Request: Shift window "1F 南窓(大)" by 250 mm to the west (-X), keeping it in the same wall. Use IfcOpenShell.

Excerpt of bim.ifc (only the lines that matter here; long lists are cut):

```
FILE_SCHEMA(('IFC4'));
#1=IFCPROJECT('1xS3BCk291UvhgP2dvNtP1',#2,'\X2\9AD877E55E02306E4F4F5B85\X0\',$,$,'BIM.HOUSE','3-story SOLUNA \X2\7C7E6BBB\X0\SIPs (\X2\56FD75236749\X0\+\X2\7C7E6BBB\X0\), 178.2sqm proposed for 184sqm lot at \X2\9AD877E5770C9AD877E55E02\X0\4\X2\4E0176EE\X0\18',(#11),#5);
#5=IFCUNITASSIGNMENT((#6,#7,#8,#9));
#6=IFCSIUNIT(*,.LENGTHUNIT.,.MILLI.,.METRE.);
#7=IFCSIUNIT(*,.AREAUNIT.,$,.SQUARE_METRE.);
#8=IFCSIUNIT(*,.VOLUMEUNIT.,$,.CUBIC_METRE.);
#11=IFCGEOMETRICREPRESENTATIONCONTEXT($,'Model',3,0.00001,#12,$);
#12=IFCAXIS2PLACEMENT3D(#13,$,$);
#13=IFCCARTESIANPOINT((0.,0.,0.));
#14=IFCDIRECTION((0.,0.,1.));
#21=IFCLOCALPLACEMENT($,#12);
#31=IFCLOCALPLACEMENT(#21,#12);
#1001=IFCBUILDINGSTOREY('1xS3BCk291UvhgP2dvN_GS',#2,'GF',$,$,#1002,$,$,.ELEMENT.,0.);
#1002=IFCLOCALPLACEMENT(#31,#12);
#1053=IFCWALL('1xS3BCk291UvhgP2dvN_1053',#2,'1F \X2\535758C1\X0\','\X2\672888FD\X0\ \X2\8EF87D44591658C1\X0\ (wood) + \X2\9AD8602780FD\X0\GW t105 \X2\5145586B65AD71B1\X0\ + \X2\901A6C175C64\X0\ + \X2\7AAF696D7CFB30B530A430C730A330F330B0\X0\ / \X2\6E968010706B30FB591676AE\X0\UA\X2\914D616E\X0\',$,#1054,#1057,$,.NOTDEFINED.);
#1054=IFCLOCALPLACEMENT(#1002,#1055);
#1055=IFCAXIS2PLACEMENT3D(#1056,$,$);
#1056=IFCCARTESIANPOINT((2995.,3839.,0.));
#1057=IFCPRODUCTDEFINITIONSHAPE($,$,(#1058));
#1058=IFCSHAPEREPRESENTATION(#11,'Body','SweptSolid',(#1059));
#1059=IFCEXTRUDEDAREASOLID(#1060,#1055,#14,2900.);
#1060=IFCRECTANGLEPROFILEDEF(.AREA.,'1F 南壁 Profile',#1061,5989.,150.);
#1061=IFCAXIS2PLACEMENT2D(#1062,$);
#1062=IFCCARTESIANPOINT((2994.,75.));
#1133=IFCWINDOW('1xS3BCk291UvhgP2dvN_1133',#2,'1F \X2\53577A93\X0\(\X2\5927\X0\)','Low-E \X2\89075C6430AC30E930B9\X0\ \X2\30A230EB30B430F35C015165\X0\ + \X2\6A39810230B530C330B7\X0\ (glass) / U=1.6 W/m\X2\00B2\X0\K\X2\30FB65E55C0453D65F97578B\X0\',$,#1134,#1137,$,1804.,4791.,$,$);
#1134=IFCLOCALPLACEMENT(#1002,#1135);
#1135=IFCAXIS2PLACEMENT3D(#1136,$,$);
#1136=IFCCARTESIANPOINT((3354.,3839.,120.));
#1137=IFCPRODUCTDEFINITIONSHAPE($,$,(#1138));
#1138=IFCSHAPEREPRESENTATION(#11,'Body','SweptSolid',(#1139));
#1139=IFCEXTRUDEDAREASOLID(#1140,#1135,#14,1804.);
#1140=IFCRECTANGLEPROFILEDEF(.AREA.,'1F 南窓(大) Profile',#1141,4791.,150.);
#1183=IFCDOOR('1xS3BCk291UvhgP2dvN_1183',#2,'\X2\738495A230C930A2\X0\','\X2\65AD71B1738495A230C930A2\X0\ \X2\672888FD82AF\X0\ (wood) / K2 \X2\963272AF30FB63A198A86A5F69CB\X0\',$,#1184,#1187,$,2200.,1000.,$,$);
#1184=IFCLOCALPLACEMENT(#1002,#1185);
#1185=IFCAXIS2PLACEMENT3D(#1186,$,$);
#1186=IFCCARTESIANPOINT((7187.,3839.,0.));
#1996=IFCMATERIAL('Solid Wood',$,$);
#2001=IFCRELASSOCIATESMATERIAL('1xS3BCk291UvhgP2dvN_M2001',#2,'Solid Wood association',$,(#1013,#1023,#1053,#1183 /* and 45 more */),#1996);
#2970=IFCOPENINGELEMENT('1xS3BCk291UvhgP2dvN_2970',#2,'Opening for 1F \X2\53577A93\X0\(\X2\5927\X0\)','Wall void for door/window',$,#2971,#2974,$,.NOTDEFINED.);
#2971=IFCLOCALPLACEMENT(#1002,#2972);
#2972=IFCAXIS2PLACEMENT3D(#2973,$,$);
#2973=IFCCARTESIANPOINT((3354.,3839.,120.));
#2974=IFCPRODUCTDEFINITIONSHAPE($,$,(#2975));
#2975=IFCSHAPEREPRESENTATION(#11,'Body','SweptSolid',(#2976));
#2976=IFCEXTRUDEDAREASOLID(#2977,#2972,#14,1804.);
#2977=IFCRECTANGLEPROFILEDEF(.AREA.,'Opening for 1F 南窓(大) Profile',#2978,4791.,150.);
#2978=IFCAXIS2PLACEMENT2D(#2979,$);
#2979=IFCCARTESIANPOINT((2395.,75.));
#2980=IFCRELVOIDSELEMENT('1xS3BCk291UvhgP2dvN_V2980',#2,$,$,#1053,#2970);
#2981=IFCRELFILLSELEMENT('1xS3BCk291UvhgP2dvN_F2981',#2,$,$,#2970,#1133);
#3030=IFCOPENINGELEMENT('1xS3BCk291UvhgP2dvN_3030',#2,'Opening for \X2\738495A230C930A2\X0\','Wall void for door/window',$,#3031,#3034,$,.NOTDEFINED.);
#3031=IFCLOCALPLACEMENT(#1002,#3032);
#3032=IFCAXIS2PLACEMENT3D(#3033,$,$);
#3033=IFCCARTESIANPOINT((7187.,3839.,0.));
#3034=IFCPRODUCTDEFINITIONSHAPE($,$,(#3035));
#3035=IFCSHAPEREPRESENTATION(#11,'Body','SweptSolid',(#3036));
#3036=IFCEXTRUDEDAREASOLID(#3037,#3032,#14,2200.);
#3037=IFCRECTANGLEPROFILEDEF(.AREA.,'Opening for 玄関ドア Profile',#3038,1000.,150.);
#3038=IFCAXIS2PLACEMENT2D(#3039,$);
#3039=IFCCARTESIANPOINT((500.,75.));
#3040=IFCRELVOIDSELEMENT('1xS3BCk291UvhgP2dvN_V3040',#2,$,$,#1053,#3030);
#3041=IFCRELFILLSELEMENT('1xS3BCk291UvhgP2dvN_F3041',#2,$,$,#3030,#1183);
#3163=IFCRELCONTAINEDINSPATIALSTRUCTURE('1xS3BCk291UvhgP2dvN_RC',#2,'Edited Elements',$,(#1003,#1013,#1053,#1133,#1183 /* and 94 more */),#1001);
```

```python
import ifcopenshell
import ifcopenshell.api.geometry
import ifcopenshell.util.placement

model = ifcopenshell.open("bim.ifc")

window = model.by_guid("1xS3BCk291UvhgP2dvN_1133")
opening = window.FillsVoids[0].RelatingOpeningElement
wall = opening.VoidsElements[0].RelatingBuildingElement

wall_matrix = ifcopenshell.util.placement.get_local_placement(wall.ObjectPlacement)
shift = wall_matrix[:3, 0] * -250.0
before = ifcopenshell.util.placement.get_local_placement(window.ObjectPlacement)[:3, 3].copy()

# The window is not placed relative to its opening, so move both.
for product in (opening, window):
    matrix = ifcopenshell.util.placement.get_local_placement(product.ObjectPlacement)
    matrix[:3, 3] += shift
    ifcopenshell.api.geometry.edit_object_placement(model, product=product, matrix=matrix, is_si=False)

after = ifcopenshell.util.placement.get_local_placement(window.ObjectPlacement)[:3, 3]
print("window moved by", (after - before).round(3) + 0.0)

model.write("bim_edited.ifc")
```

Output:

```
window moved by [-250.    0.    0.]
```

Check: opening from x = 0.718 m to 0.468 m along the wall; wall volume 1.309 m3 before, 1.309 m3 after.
